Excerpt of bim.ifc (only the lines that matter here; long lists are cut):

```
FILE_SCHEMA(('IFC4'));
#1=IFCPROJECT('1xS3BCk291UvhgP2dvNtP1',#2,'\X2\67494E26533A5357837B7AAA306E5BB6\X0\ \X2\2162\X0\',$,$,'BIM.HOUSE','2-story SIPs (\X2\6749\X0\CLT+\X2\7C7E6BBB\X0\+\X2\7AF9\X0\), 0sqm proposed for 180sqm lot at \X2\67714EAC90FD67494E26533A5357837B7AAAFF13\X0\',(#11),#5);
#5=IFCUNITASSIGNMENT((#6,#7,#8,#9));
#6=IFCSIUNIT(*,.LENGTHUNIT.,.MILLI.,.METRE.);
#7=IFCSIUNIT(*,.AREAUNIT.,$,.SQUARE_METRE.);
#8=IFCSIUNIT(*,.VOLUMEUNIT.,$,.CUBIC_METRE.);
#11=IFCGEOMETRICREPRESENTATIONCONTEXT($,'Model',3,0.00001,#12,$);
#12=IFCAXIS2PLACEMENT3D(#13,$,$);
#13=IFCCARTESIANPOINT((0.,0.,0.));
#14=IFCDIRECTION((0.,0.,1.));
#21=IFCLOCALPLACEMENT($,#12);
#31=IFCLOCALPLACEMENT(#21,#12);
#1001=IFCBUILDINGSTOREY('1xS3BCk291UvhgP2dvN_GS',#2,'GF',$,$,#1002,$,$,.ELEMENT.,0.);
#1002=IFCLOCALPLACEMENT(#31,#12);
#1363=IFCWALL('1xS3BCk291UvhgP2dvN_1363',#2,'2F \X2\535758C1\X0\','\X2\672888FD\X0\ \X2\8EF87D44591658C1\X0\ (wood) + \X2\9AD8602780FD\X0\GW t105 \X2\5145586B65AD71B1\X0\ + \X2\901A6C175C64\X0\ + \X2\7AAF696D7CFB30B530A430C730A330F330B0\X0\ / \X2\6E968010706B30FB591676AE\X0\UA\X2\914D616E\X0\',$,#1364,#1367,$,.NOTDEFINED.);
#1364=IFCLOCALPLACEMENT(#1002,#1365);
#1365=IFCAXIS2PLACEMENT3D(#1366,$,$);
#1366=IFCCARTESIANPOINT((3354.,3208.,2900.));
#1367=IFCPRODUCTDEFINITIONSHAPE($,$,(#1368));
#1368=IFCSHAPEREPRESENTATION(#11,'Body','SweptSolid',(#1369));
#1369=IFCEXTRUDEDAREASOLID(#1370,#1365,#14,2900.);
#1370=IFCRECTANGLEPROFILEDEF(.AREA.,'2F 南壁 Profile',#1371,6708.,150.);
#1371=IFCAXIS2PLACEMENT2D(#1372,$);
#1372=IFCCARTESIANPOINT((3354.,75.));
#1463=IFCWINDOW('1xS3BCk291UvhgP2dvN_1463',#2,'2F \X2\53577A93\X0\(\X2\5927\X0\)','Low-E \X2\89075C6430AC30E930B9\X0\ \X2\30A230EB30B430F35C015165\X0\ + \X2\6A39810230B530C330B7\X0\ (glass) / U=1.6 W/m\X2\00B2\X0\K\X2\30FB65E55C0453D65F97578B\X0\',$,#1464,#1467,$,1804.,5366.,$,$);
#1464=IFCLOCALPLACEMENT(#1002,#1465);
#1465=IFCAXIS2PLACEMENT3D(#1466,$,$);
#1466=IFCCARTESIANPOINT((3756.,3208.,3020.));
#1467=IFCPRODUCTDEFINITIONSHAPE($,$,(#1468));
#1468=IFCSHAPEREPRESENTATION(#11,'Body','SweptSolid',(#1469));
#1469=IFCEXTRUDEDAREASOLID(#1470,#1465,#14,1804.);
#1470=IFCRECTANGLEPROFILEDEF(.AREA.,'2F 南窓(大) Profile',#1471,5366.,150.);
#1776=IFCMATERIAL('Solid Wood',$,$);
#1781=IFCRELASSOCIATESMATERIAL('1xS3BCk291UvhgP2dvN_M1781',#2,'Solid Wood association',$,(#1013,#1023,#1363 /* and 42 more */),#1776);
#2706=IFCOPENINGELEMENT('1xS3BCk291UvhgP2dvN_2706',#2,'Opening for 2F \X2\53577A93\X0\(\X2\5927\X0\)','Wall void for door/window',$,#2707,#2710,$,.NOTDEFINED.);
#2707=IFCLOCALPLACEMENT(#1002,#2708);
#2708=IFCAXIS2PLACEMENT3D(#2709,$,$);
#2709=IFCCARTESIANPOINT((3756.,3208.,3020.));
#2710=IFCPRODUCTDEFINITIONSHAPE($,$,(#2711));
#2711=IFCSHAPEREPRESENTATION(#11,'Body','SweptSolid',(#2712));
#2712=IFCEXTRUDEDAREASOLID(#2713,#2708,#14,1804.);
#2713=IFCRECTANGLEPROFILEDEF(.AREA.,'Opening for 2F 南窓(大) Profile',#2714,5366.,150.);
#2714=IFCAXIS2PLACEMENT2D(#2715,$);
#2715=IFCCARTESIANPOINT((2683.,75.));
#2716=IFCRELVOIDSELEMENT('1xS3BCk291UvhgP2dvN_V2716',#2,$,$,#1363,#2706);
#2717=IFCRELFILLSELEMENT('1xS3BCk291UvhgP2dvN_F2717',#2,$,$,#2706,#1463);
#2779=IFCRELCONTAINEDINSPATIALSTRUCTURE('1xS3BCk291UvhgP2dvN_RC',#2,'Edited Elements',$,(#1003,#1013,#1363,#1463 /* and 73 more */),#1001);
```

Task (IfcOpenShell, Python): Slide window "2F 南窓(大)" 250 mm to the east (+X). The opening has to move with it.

```python
import ifcopenshell
import ifcopenshell.api.geometry
import ifcopenshell.util.placement
import ifcopenshell.util.unit

model = ifcopenshell.open("bim.ifc")
unit_scale = ifcopenshell.util.unit.calculate_unit_scale(model)

window = model.by_guid("1xS3BCk291UvhgP2dvN_1463")
opening = window.FillsVoids[0].RelatingOpeningElement
wall = opening.VoidsElements[0].RelatingBuildingElement

wall_matrix = ifcopenshell.util.placement.get_local_placement(wall.ObjectPlacement)
shift = wall_matrix[:3, 0] * 0.25 / unit_scale
before = ifcopenshell.util.placement.get_local_placement(window.ObjectPlacement)[:3, 3].copy()

# The window is not placed relative to its opening, so move both.
for product in (opening, window):
    matrix = ifcopenshell.util.placement.get_local_placement(product.ObjectPlacement)
    matrix[:3, 3] += shift
    ifcopenshell.api.geometry.edit_object_placement(model, product=product, matrix=matrix, is_si=False)

after = ifcopenshell.util.placement.get_local_placement(window.ObjectPlacement)[:3, 3]
print("window moved by", (after - before).round(3) + 0.0)

model.write("bim_edited.ifc")
```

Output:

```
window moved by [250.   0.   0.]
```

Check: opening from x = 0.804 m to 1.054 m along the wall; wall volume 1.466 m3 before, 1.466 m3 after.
